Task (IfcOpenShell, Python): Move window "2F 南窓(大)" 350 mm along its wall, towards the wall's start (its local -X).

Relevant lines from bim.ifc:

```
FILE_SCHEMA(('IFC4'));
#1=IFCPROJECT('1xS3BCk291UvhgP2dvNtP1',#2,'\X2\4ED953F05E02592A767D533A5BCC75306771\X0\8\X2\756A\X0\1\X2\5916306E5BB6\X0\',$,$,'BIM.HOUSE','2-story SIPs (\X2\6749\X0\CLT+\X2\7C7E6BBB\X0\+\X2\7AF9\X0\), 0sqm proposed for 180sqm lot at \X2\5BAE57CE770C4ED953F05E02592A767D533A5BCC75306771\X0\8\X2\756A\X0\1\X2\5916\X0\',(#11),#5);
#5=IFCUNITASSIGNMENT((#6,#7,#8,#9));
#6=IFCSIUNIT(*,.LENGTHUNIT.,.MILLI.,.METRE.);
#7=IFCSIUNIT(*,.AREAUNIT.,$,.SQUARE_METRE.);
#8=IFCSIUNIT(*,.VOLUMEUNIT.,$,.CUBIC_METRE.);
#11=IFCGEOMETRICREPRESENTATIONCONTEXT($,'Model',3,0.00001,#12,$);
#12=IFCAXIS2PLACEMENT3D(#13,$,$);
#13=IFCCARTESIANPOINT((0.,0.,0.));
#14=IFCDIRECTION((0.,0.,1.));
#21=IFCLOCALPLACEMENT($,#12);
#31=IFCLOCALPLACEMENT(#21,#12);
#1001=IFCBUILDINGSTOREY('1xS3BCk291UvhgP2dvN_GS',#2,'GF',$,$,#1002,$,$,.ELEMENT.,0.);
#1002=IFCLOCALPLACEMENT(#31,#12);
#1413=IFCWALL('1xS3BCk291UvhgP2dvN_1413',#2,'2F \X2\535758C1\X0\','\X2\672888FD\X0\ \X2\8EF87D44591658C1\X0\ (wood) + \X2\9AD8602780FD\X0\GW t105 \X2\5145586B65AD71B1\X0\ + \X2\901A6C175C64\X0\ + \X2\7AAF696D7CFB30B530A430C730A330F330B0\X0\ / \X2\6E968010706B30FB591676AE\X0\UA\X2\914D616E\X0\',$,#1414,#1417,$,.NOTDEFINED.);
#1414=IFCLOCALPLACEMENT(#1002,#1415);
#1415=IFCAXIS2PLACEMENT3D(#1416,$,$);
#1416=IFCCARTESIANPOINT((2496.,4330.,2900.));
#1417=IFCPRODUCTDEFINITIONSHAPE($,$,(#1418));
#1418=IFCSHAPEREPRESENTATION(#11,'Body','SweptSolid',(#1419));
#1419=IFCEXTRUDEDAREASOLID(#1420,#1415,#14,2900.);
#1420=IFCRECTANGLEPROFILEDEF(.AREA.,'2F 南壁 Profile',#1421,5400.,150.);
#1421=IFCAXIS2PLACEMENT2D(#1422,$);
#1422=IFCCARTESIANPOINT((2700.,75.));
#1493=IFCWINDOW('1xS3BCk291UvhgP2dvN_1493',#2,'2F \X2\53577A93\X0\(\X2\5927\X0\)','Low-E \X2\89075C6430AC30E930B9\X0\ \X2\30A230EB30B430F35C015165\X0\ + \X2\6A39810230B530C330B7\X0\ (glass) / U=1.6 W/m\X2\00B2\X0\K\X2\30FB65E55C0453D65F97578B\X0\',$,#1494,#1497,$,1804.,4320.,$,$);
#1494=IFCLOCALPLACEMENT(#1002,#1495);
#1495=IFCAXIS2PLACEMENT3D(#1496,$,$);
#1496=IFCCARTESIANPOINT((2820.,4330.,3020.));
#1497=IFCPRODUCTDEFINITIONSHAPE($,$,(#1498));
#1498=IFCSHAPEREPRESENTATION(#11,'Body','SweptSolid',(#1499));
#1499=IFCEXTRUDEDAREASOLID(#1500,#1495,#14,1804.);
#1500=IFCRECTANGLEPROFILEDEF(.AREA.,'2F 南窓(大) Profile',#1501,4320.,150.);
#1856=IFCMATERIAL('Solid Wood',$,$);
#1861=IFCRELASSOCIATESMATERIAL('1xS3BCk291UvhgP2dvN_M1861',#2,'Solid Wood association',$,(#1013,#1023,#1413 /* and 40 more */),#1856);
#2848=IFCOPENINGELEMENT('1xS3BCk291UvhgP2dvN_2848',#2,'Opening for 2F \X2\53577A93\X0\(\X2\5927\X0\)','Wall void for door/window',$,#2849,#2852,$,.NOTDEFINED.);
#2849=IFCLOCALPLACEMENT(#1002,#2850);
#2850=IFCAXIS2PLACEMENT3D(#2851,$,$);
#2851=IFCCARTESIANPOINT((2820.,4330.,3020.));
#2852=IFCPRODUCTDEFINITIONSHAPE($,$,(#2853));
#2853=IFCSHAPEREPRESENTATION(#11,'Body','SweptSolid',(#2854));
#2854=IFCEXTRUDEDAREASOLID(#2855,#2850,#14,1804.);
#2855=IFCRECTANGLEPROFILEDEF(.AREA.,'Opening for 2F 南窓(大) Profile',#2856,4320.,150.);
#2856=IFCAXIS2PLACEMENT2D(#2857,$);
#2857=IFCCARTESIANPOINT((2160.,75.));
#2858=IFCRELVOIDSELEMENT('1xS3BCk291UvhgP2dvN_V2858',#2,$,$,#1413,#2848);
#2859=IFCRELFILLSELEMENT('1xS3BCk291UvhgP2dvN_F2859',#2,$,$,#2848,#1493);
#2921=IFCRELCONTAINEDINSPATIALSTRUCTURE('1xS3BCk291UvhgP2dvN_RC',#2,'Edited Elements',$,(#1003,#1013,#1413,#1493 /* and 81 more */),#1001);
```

```python
import ifcopenshell
import ifcopenshell.api.geometry
import ifcopenshell.util.placement

model = ifcopenshell.open("bim.ifc")

window = model.by_guid("1xS3BCk291UvhgP2dvN_1493")
opening = window.FillsVoids[0].RelatingOpeningElement
wall = opening.VoidsElements[0].RelatingBuildingElement

wall_matrix = ifcopenshell.util.placement.get_local_placement(wall.ObjectPlacement)
shift = wall_matrix[:3, 0] * -350.0
before = ifcopenshell.util.placement.get_local_placement(window.ObjectPlacement)[:3, 3].copy()

# The window is not placed relative to its opening, so move both.
for product in (opening, window):
    matrix = ifcopenshell.util.placement.get_local_placement(product.ObjectPlacement)
    matrix[:3, 3] += shift
    ifcopenshell.api.geometry.edit_object_placement(model, product=product, matrix=matrix, is_si=False)

after = ifcopenshell.util.placement.get_local_placement(window.ObjectPlacement)[:3, 3]
print("window moved by", (after - before).round(3) + 0.0)

model.write("bim_v2.ifc")
```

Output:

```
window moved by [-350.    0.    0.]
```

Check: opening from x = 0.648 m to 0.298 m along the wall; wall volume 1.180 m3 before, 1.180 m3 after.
